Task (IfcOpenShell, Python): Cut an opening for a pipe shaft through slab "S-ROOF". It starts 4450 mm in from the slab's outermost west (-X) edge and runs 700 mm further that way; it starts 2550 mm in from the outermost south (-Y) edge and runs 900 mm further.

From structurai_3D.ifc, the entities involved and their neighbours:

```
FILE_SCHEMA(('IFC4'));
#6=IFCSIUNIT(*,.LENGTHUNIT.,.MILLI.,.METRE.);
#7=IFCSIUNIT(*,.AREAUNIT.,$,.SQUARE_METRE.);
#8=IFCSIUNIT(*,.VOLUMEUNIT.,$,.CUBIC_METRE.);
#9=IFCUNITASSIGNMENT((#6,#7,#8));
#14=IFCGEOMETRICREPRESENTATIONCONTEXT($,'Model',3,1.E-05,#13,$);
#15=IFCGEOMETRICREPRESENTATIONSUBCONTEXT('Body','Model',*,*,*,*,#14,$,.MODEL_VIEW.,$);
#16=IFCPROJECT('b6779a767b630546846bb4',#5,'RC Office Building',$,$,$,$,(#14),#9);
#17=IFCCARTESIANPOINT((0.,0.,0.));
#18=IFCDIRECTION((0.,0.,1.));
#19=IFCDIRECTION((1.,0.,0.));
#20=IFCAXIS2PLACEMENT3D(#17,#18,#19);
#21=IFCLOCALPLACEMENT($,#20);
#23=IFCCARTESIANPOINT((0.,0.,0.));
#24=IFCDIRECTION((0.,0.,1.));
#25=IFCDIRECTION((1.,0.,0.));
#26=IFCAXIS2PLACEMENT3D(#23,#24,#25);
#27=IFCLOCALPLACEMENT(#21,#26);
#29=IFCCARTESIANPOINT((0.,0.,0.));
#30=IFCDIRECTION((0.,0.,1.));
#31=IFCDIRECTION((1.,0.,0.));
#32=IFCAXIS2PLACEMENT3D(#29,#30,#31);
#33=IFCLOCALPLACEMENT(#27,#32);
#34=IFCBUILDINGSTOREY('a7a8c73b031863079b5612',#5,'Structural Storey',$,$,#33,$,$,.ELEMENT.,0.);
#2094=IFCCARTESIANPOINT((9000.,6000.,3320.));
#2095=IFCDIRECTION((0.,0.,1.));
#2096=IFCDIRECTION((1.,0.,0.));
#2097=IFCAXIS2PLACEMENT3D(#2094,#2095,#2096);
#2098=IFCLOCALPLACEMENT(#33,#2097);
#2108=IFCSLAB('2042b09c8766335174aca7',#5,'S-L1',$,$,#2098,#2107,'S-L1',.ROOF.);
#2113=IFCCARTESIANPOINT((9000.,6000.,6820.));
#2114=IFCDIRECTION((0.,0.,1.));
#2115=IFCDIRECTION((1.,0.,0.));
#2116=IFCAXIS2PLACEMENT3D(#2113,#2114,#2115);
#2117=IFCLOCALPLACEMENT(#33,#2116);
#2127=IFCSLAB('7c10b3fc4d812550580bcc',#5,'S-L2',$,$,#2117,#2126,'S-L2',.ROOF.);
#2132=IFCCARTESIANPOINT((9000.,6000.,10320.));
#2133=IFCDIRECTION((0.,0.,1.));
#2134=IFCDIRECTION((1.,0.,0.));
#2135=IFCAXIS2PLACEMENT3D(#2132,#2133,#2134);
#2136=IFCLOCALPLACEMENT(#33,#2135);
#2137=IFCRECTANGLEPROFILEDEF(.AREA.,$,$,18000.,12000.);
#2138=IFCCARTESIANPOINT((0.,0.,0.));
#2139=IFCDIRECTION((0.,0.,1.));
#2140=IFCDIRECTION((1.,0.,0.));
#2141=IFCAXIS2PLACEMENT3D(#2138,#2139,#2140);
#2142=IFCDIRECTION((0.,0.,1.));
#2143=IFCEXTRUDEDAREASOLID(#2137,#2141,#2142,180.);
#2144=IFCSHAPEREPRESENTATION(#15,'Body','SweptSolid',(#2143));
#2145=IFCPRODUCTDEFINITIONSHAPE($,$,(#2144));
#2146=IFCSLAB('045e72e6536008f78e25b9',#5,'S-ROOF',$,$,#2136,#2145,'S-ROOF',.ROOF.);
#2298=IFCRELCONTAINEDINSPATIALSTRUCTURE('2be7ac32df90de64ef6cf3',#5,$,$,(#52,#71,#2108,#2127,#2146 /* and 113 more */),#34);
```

```python
import numpy as np
import ifcopenshell
import ifcopenshell.api.feature
import ifcopenshell.api.geometry
import ifcopenshell.api.root
import ifcopenshell.geom
import ifcopenshell.util.placement
import ifcopenshell.util.representation
import ifcopenshell.util.shape
import ifcopenshell.util.unit

model = ifcopenshell.open("structurai_3D.ifc")
unit_scale = ifcopenshell.util.unit.calculate_unit_scale(model)
settings = ifcopenshell.geom.settings()


def volume(element):
    """Net volume in cubic metres, openings subtracted."""
    shape = ifcopenshell.geom.create_shape(settings, element)
    return ifcopenshell.util.shape.get_volume(shape.geometry)


slab = model.by_guid("045e72e6536008f78e25b9")
before = volume(slab)

# Extent in the slab's own axes, in metres. The edges named are its -X and -Y sides.
slab_shape = ifcopenshell.geom.create_shape(settings, slab)
vertices = ifcopenshell.util.shape.get_vertices(slab_shape.geometry)
x_min, y_min, bottom = vertices.min(axis=0)
top = vertices[:, 2].max()

opening = ifcopenshell.api.root.create_entity(model, ifc_class="IfcOpeningElement", name="Pipe shaft opening", predefined_type="OPENING")
context = ifcopenshell.util.representation.get_context(model, "Model", "Body", "MODEL_VIEW")
width, depth = 0.7, 0.9
outline = [(0.0, 0.0), (width, 0.0), (width, depth), (0.0, depth), (0.0, 0.0)]
# Overshoot both faces by 50 mm so the cut is clean.
shape = ifcopenshell.api.geometry.add_slab_representation(
    model, context=context, depth=top - bottom + 0.1, polyline=outline
)
ifcopenshell.api.geometry.assign_representation(model, product=opening, representation=shape)

matrix = ifcopenshell.util.placement.get_local_placement(slab.ObjectPlacement)
matrix[:, 3] = matrix @ np.append(np.array([x_min + 4.45, y_min + 2.55, bottom - 0.05]) / unit_scale, 1.0)
ifcopenshell.api.geometry.edit_object_placement(model, product=opening, matrix=matrix, is_si=False)
ifcopenshell.api.feature.add_feature(model, feature=opening, element=slab)

after = volume(slab)

print(f"slab volume {before:.3f} -> {after:.3f} m3")

model.write("structurai_3D_v2.ifc")
```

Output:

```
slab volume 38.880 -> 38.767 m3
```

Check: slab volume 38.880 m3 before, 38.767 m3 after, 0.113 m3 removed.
